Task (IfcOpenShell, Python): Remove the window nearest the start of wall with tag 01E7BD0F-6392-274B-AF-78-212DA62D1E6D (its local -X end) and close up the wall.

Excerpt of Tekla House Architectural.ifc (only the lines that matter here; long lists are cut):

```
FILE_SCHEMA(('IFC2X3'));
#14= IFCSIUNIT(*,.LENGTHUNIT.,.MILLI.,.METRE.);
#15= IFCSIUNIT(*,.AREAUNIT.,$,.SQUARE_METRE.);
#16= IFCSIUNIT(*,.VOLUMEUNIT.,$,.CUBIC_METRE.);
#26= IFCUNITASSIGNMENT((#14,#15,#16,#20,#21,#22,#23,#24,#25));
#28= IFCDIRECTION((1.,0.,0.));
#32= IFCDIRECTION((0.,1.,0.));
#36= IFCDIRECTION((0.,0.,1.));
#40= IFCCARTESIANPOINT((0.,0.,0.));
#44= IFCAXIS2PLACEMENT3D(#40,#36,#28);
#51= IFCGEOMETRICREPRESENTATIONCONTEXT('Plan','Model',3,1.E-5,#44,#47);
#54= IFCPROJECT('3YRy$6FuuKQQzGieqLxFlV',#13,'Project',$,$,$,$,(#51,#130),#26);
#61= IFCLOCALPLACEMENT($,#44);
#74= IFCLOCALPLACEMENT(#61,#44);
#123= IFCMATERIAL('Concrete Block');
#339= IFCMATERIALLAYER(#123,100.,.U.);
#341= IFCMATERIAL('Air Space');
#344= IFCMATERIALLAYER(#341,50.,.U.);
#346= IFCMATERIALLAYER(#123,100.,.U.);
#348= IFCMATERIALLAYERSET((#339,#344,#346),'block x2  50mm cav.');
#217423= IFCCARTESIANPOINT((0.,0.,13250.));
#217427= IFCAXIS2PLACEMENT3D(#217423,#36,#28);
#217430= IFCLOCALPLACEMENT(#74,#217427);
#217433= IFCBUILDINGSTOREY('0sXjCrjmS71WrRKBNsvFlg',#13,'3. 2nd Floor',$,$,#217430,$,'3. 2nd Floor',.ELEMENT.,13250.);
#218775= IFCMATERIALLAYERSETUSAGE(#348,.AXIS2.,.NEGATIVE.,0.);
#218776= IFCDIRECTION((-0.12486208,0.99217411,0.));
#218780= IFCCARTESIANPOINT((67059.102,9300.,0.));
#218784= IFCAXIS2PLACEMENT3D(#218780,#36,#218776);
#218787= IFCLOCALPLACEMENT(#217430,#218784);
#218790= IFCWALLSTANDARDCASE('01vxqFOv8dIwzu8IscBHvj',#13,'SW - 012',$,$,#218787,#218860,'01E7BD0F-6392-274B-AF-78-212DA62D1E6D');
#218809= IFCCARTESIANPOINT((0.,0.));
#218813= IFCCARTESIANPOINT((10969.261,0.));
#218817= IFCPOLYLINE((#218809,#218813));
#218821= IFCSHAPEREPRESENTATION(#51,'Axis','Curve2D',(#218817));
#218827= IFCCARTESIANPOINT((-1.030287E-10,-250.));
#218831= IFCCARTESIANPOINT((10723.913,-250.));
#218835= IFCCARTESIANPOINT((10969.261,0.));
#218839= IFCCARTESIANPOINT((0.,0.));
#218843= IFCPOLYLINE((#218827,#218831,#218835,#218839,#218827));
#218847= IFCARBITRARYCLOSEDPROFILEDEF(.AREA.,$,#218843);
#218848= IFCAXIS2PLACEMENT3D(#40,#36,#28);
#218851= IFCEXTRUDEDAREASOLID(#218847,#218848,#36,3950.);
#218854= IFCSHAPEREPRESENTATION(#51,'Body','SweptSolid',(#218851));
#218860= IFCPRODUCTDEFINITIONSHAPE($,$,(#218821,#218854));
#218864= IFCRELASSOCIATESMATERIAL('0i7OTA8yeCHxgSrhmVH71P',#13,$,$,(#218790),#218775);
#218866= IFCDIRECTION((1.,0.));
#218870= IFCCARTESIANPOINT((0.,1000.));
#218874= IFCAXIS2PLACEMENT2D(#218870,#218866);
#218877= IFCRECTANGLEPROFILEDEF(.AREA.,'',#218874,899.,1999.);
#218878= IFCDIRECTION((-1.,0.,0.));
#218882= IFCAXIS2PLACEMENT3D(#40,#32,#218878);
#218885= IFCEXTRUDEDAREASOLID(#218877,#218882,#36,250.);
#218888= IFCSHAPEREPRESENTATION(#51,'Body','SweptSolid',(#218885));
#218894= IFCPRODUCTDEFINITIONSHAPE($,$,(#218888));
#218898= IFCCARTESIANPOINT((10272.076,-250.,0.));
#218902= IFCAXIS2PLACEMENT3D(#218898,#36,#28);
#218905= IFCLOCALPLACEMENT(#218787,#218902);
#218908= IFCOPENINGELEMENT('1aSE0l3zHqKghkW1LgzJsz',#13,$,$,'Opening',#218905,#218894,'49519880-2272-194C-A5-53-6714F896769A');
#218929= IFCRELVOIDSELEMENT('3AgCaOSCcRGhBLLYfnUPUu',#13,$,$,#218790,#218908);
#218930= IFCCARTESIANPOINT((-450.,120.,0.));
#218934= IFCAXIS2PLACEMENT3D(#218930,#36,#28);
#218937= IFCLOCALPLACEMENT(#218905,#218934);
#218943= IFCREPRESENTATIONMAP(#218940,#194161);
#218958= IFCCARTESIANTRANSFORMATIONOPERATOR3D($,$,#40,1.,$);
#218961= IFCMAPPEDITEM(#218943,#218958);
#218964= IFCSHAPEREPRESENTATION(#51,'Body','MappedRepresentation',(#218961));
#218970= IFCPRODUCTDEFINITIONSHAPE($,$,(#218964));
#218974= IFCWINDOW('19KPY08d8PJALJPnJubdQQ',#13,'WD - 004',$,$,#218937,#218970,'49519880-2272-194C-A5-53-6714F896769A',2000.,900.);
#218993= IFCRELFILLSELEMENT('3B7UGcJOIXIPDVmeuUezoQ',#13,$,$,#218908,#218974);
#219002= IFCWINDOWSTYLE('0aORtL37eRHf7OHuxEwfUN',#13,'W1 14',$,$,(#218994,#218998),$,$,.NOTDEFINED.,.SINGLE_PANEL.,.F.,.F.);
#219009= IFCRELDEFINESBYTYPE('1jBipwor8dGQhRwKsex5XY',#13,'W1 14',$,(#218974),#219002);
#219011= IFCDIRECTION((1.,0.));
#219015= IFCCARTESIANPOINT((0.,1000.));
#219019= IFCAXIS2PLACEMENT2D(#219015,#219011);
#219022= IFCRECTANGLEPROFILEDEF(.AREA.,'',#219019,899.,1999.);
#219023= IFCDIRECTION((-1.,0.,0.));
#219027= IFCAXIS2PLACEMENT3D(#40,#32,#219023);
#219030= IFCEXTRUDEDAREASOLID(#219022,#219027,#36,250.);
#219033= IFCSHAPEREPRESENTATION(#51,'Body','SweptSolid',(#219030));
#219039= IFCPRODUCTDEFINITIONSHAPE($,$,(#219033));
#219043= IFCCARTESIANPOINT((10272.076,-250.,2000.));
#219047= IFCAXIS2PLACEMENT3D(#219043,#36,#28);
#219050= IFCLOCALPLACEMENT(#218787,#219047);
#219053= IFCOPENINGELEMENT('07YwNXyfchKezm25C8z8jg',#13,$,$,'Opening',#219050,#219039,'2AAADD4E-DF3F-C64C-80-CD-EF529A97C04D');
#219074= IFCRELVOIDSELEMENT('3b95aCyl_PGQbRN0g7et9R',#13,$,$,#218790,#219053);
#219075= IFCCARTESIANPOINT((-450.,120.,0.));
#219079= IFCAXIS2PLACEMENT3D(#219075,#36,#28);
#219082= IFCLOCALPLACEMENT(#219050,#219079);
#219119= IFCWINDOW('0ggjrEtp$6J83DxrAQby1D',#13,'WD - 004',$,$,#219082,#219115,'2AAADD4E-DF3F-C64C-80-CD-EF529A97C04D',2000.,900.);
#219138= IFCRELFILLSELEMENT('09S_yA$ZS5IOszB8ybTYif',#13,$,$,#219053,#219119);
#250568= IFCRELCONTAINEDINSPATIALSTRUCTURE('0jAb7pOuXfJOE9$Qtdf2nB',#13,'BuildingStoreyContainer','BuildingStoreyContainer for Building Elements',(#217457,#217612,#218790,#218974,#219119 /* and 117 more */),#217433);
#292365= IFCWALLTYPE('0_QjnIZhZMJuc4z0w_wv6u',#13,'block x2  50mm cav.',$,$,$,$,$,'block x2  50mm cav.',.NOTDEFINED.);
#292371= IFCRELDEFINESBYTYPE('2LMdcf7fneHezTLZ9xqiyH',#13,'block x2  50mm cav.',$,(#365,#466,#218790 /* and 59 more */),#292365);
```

```python
import ifcopenshell
import ifcopenshell.api.feature
import ifcopenshell.api.root
import ifcopenshell.geom
import ifcopenshell.util.shape

model = ifcopenshell.open("Tekla House Architectural.ifc")
settings = ifcopenshell.geom.settings()


def volume(element):
    """Net volume in cubic metres, openings subtracted."""
    shape = ifcopenshell.geom.create_shape(settings, element)
    return ifcopenshell.util.shape.get_volume(shape.geometry)


window = model.by_guid("19KPY08d8PJALJPnJubdQQ")
opening = window.FillsVoids[0].RelatingOpeningElement
wall = opening.VoidsElements[0].RelatingBuildingElement
before = volume(wall)

ifcopenshell.api.root.remove_product(model, product=window)
ifcopenshell.api.feature.remove_feature(model, feature=opening)

after = volume(wall)

print(f"wall volume {before:.3f} -> {after:.3f} m3")

model.write("Tekla House Architectural-out.ifc")
```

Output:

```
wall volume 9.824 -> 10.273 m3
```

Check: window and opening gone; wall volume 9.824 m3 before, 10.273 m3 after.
